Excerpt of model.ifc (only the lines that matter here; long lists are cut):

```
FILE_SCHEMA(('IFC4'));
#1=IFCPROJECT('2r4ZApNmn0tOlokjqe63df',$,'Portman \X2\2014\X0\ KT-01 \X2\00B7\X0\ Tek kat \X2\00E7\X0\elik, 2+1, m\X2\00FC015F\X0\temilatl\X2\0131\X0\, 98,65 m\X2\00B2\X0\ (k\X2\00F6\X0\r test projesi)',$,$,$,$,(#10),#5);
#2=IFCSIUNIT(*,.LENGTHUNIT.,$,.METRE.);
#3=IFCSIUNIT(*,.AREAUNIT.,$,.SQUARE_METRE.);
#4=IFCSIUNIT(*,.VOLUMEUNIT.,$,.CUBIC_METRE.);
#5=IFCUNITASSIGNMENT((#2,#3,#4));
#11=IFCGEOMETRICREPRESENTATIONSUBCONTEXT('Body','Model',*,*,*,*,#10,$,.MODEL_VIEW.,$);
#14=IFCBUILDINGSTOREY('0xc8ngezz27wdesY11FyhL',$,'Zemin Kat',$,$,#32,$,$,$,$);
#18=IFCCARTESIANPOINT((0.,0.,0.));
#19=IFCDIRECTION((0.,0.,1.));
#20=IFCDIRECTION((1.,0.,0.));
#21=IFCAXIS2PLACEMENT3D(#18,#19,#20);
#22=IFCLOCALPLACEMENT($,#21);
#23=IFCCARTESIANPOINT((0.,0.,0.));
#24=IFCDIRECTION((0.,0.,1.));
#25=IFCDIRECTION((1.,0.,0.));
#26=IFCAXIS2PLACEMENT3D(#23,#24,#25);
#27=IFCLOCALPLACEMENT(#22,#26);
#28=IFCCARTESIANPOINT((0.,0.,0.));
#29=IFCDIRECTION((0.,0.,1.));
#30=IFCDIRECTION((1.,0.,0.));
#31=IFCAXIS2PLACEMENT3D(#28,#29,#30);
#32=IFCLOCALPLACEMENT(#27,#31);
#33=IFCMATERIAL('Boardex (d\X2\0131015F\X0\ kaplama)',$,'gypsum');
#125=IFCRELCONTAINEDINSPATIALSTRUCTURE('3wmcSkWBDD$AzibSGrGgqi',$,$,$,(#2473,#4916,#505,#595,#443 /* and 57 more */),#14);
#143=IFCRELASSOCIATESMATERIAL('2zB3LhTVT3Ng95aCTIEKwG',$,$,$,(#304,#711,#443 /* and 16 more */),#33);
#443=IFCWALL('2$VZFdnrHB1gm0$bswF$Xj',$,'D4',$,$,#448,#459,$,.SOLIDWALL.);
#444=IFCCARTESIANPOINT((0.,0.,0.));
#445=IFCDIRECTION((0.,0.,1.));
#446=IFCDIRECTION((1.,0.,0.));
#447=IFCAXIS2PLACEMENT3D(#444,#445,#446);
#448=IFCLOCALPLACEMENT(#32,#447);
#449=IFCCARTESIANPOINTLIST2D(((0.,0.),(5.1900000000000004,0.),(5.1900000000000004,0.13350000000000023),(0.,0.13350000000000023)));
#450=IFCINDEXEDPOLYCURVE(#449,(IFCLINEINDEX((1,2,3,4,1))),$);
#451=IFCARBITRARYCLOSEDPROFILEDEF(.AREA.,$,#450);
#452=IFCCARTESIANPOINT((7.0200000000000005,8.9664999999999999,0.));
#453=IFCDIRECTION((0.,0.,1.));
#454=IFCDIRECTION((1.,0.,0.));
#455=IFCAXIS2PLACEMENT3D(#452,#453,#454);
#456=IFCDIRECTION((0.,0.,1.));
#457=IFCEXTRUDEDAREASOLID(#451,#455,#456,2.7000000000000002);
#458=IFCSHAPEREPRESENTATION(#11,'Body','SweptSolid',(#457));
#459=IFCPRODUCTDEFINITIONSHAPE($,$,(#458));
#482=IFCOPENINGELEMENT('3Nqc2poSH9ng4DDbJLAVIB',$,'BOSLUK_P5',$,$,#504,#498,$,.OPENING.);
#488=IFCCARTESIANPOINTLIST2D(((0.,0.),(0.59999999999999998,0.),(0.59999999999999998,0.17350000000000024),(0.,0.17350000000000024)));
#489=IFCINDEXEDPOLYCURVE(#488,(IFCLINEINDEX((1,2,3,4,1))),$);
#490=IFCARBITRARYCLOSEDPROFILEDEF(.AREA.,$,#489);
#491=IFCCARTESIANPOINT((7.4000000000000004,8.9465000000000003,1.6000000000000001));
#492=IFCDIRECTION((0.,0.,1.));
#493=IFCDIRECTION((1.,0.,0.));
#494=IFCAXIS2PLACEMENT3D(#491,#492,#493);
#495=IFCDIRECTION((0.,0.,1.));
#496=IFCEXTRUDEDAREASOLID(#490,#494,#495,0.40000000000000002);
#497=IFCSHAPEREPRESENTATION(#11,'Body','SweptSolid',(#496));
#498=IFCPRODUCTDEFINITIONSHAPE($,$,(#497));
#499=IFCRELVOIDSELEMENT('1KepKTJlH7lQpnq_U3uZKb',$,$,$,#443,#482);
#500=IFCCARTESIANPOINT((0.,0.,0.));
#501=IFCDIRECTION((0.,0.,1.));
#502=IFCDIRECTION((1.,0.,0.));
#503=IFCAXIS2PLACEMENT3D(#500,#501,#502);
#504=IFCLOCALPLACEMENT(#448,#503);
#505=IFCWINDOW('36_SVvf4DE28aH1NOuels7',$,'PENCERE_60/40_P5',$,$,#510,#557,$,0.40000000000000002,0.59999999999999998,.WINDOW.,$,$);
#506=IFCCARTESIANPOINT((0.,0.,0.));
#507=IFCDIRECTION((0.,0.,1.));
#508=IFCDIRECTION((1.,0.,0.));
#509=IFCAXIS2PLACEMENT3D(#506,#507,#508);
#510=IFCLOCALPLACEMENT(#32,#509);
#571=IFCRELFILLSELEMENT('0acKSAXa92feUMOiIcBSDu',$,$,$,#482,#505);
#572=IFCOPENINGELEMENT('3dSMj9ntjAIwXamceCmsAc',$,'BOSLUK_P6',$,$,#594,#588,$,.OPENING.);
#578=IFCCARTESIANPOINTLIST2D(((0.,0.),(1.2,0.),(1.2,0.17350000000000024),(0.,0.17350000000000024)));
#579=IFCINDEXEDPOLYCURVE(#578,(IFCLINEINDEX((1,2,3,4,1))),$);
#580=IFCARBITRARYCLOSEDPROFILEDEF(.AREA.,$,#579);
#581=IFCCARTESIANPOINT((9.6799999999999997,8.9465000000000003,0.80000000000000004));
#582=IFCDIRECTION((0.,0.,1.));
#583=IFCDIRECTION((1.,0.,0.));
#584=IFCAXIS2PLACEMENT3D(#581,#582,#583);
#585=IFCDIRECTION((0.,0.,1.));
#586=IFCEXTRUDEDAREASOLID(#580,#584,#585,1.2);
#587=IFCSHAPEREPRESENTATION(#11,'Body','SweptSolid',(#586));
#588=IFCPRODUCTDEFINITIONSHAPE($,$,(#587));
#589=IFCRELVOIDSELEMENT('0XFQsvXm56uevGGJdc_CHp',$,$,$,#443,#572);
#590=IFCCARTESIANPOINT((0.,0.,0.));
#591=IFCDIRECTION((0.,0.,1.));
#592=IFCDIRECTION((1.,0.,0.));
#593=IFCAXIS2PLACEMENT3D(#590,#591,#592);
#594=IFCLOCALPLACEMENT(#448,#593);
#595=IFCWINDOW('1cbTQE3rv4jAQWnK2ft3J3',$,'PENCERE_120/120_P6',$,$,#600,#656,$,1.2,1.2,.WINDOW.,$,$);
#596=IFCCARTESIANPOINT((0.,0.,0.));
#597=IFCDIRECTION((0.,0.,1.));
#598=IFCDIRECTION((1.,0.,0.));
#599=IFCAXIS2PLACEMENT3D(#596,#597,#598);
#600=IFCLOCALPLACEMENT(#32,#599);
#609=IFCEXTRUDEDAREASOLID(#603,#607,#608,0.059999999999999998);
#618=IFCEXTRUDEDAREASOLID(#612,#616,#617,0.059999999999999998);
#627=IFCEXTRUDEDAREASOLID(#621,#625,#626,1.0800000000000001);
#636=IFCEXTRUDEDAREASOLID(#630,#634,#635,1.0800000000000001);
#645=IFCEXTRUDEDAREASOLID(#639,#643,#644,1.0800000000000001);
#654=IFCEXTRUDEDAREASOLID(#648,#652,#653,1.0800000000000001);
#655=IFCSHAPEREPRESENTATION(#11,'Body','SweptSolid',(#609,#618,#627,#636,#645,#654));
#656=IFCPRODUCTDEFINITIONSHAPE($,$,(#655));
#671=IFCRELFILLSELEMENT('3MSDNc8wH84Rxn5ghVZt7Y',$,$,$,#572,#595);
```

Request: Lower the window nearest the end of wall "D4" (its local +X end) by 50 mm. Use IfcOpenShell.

```python
import numpy as np
import ifcopenshell
import ifcopenshell.api.geometry
import ifcopenshell.util.placement
import ifcopenshell.util.unit

model = ifcopenshell.open("model.ifc")
unit_scale = ifcopenshell.util.unit.calculate_unit_scale(model)

window = model.by_guid("1cbTQE3rv4jAQWnK2ft3J3")
opening = window.FillsVoids[0].RelatingOpeningElement
dz = -0.05 / unit_scale

shift = np.array([0.0, 0.0, dz])
# The window is not placed relative to its opening, so move both.
for product in (opening, window):
    matrix = ifcopenshell.util.placement.get_local_placement(product.ObjectPlacement)
    matrix[:3, 3] += shift
    ifcopenshell.api.geometry.edit_object_placement(model, product=product, matrix=matrix, is_si=False)

print(f"moved by {dz * unit_scale:+.3f} m")

model.write("model_rev.ifc")
```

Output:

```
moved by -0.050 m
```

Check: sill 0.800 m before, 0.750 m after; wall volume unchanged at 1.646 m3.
